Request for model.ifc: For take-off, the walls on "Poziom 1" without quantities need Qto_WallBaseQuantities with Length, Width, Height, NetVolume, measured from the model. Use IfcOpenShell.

First a look at what the model holds.

```python
import ifcopenshell
import ifcopenshell.util.element
import ifcopenshell.util.unit

model = ifcopenshell.open("model.ifc")
print(model.schema)
for unit_type in ("LENGTHUNIT", "AREAUNIT", "VOLUMEUNIT"):
    print(unit_type, ifcopenshell.util.unit.calculate_unit_scale(model, unit_type))
storey = next(s for s in model.by_type("IfcBuildingStorey") if s.Name == "Poziom 1")
walls = [e for e in ifcopenshell.util.element.get_decomposition(storey) if e.is_a("IfcWall")]
for e in sorted(walls, key=lambda e: e.id()):
    print(e.id(), e.is_a(), e.Name, list(ifcopenshell.util.element.get_psets(e, qtos_only=True)), sep=" | ")
```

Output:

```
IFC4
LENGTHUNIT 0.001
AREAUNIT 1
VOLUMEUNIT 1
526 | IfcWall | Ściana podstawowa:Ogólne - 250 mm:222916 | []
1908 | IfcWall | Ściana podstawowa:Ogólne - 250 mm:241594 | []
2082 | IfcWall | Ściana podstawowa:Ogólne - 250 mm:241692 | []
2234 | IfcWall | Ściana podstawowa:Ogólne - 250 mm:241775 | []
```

```python
import ifcopenshell
import ifcopenshell.api.pset
import ifcopenshell.geom
import ifcopenshell.util.element
import ifcopenshell.util.shape
import ifcopenshell.util.unit

model = ifcopenshell.open("model.ifc")
unit_scale = ifcopenshell.util.unit.calculate_unit_scale(model)
volume_scale = ifcopenshell.util.unit.calculate_unit_scale(model, "VOLUMEUNIT")
settings = ifcopenshell.geom.settings()

storey = next(s for s in model.by_type("IfcBuildingStorey") if s.Name == "Poziom 1")
walls = [e for e in ifcopenshell.util.element.get_decomposition(storey) if e.is_a("IfcWall")]

for e in sorted(walls, key=lambda e: e.id()):
    if ifcopenshell.util.element.get_psets(e, qtos_only=True, should_inherit=False):
        continue
    # Geometry comes back in metres, in the element's own axes.
    shape = ifcopenshell.geom.create_shape(settings, e)
    values = {
        "Length": ifcopenshell.util.shape.get_x(shape.geometry) / unit_scale,
        "Width": ifcopenshell.util.shape.get_y(shape.geometry) / unit_scale,
        "Height": ifcopenshell.util.shape.get_z(shape.geometry) / unit_scale,
        "NetVolume": ifcopenshell.util.shape.get_volume(shape.geometry) / volume_scale,
    }
    qto = ifcopenshell.api.pset.add_qto(model, product=e, name="Qto_WallBaseQuantities")
    ifcopenshell.api.pset.edit_qto(model, qto=qto, properties=values)
    print(e.id(), {k: round(v, 3) for k, v in values.items()})

model.write("model-out.ifc")
```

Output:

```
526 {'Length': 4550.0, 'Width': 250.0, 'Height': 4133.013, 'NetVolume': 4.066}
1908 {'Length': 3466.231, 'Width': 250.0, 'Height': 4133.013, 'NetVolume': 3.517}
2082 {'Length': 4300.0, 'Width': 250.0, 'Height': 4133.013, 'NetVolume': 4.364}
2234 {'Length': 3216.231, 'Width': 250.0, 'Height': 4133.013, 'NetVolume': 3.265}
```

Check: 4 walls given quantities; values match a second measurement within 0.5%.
